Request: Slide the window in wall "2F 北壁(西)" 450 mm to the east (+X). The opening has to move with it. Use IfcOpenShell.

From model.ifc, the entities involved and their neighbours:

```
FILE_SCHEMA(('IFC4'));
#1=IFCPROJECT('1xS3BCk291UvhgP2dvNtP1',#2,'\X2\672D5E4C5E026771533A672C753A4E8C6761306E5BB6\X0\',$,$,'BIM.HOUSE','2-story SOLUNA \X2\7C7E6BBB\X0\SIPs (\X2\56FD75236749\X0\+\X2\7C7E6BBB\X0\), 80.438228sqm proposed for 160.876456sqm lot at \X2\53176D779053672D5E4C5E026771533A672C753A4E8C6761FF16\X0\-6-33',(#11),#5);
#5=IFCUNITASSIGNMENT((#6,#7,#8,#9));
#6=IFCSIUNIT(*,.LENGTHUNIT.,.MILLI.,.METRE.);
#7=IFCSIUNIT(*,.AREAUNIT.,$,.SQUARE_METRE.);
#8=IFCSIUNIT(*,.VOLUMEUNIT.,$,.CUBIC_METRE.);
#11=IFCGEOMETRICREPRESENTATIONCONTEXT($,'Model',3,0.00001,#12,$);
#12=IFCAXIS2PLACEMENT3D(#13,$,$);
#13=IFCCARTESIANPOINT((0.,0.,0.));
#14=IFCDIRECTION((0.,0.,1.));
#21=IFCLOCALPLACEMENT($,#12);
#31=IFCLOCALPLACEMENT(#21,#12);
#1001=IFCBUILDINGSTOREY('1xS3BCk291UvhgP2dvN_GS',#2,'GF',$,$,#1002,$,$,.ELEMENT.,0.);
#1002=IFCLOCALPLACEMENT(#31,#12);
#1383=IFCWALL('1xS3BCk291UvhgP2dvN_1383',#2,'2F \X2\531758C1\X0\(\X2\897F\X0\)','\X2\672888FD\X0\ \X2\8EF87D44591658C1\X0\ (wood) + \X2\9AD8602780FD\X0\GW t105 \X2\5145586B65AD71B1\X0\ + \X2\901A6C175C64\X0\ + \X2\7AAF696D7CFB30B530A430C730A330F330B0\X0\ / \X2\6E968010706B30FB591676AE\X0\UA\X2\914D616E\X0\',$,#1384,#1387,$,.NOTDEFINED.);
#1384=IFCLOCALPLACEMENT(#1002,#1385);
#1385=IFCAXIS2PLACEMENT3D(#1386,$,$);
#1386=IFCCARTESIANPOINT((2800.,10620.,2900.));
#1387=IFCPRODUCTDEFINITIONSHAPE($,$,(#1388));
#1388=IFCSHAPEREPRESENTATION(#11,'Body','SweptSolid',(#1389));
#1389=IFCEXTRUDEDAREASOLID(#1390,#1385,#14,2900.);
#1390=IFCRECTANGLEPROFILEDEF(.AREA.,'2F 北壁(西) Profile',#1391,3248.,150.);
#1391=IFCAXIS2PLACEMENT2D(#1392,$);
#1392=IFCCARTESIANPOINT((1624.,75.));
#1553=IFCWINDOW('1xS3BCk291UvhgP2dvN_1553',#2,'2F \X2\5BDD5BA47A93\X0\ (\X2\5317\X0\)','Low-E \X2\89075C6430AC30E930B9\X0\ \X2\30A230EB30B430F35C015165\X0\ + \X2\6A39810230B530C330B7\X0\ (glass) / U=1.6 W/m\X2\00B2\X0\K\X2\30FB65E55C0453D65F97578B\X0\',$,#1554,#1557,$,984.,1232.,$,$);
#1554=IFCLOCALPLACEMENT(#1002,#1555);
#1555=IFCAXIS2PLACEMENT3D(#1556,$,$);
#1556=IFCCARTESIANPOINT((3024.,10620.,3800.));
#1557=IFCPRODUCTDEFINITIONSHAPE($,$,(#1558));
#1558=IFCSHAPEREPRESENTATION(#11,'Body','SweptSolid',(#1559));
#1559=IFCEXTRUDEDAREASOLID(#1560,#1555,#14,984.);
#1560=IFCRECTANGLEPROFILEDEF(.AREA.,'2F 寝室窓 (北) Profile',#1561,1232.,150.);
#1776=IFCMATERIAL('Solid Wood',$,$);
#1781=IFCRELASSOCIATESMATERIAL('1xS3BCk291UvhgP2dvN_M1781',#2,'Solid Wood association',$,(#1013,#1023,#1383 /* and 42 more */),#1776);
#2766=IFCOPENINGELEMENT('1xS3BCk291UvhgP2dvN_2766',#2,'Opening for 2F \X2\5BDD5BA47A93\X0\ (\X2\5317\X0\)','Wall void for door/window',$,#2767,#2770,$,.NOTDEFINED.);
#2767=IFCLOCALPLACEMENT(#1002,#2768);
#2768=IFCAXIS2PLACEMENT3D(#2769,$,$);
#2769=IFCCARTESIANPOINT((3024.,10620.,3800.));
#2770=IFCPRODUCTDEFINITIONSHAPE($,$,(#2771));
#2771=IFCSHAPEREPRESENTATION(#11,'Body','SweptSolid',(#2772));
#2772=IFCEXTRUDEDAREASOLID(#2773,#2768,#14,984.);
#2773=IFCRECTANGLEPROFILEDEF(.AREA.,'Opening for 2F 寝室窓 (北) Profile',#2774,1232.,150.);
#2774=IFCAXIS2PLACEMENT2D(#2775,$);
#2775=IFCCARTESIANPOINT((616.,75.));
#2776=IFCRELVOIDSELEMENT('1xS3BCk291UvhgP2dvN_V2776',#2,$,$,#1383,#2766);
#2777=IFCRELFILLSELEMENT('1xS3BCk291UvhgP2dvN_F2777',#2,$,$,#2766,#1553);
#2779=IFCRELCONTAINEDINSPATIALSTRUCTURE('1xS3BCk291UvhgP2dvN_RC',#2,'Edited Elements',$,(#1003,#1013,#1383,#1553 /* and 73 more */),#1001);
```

```python
import ifcopenshell
import ifcopenshell.api.geometry
import ifcopenshell.util.placement
import ifcopenshell.util.unit

model = ifcopenshell.open("model.ifc")
unit_scale = ifcopenshell.util.unit.calculate_unit_scale(model)

window = model.by_id(1553)
opening = window.FillsVoids[0].RelatingOpeningElement
wall = opening.VoidsElements[0].RelatingBuildingElement

wall_matrix = ifcopenshell.util.placement.get_local_placement(wall.ObjectPlacement)
shift = wall_matrix[:3, 0] * 0.45 / unit_scale
before = ifcopenshell.util.placement.get_local_placement(window.ObjectPlacement)[:3, 3].copy()

# The window is not placed relative to its opening, so move both.
for product in (opening, window):
    matrix = ifcopenshell.util.placement.get_local_placement(product.ObjectPlacement)
    matrix[:3, 3] += shift
    ifcopenshell.api.geometry.edit_object_placement(model, product=product, matrix=matrix, is_si=False)

after = ifcopenshell.util.placement.get_local_placement(window.ObjectPlacement)[:3, 3]
print("window moved by", (after - before).round(3) + 0.0)

model.write("model_rev.ifc")
```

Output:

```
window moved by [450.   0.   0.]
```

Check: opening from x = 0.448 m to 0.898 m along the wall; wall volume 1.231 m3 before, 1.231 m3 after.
